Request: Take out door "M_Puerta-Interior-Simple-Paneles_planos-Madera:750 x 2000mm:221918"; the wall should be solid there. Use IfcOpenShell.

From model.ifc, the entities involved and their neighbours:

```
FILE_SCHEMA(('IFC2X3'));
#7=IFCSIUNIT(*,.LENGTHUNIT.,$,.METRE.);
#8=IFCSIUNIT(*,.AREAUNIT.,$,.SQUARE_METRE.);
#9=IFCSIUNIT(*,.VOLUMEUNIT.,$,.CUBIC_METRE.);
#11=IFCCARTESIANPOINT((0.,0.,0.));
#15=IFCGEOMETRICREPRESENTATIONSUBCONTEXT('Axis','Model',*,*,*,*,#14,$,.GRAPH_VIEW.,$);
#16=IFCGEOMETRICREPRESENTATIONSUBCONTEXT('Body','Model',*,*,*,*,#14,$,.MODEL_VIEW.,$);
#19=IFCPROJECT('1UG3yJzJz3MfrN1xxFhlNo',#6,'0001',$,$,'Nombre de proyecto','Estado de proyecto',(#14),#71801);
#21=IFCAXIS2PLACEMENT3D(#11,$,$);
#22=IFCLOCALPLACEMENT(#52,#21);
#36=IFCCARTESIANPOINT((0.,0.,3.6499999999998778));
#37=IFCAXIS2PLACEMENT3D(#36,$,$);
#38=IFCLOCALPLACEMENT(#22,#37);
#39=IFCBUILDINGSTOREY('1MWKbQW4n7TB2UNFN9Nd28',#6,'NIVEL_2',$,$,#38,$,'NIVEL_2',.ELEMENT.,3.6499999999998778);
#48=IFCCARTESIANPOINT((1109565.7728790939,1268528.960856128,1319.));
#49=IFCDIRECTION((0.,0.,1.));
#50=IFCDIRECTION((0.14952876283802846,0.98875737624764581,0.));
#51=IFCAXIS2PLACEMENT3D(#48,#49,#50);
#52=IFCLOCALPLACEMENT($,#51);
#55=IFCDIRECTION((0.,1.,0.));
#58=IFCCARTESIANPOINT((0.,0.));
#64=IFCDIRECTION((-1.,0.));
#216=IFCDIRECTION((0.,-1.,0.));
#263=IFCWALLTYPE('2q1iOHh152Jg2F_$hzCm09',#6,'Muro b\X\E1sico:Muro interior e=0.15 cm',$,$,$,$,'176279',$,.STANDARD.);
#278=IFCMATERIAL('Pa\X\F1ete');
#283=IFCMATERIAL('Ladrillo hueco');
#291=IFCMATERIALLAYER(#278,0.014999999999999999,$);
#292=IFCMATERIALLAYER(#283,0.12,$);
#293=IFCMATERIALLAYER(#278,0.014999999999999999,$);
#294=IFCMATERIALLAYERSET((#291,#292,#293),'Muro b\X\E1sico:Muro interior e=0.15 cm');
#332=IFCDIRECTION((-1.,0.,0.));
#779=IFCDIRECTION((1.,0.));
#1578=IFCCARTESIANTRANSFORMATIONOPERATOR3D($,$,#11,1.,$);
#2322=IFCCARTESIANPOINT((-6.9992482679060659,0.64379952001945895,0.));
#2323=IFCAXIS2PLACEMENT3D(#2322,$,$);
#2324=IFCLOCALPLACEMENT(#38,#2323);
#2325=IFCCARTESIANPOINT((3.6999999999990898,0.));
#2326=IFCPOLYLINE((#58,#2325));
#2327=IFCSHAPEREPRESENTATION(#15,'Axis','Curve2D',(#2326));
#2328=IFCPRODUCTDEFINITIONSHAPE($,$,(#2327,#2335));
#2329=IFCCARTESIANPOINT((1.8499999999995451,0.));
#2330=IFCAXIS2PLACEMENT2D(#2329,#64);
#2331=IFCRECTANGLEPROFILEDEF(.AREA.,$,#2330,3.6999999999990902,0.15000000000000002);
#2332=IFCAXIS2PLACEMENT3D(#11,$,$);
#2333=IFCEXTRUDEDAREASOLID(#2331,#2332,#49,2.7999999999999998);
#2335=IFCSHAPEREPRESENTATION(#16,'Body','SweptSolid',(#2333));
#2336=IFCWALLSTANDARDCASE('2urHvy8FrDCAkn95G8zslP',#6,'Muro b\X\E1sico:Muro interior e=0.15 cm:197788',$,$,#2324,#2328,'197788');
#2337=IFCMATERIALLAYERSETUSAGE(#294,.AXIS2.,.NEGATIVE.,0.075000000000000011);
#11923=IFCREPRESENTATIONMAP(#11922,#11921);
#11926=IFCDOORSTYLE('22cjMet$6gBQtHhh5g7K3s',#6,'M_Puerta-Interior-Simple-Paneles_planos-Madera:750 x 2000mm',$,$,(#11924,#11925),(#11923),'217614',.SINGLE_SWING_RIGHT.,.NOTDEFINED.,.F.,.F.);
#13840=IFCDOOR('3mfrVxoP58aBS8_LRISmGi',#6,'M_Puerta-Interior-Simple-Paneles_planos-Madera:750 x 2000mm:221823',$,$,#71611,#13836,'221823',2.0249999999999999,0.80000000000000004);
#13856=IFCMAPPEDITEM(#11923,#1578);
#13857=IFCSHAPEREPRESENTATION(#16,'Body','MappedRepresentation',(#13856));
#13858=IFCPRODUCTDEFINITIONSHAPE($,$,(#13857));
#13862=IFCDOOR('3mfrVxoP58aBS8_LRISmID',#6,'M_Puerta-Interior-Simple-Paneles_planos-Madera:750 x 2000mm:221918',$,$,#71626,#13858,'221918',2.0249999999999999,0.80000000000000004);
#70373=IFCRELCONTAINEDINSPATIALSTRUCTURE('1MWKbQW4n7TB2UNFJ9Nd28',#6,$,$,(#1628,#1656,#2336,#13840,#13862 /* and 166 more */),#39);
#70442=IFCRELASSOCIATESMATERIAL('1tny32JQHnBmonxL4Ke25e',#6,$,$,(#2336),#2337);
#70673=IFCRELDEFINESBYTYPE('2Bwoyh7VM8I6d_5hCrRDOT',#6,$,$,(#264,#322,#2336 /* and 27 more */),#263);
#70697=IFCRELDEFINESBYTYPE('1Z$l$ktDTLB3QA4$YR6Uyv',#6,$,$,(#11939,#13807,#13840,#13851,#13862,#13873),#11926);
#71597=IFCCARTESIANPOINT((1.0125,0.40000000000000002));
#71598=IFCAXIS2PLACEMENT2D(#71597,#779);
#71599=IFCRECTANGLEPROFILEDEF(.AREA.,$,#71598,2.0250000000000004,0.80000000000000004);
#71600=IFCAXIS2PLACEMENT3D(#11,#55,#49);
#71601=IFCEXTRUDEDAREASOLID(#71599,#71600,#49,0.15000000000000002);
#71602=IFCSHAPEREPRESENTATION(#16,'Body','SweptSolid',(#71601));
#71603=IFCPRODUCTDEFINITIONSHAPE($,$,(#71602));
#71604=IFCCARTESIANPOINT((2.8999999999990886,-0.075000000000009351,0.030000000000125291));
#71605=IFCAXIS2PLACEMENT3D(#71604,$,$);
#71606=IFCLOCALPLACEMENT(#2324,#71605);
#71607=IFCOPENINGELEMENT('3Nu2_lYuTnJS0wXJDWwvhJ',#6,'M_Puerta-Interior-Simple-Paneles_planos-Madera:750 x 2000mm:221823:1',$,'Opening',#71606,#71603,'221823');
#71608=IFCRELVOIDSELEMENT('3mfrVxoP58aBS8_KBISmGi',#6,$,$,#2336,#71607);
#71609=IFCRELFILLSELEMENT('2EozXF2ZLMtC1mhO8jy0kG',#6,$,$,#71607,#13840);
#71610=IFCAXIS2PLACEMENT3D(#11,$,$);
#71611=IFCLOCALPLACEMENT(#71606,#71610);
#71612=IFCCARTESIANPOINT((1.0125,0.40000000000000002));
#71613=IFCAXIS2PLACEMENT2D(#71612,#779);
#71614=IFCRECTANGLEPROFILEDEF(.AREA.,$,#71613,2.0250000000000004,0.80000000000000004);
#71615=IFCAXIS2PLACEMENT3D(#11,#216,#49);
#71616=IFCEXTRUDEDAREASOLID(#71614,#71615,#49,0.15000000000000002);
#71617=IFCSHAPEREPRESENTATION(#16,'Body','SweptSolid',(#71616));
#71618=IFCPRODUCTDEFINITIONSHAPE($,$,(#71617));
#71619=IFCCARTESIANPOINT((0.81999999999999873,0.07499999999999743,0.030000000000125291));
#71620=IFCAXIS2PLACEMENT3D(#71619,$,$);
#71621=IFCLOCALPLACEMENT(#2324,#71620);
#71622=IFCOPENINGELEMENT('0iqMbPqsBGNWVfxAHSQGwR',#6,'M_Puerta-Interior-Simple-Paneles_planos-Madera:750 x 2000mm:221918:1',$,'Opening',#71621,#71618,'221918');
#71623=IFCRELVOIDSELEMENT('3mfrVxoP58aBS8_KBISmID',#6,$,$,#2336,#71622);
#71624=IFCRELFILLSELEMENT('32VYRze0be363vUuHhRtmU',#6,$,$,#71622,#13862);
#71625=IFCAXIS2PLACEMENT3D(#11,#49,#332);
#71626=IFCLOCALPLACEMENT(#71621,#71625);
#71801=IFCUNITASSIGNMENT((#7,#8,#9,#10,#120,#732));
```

```python
import ifcopenshell
import ifcopenshell.api.feature
import ifcopenshell.api.root
import ifcopenshell.geom
import ifcopenshell.util.shape

model = ifcopenshell.open("model.ifc")
settings = ifcopenshell.geom.settings()


def volume(element):
    """Net volume in cubic metres, openings subtracted."""
    shape = ifcopenshell.geom.create_shape(settings, element)
    return ifcopenshell.util.shape.get_volume(shape.geometry)


door = model.by_guid("3mfrVxoP58aBS8_LRISmID")
opening = door.FillsVoids[0].RelatingOpeningElement
wall = opening.VoidsElements[0].RelatingBuildingElement
before = volume(wall)

ifcopenshell.api.root.remove_product(model, product=door)
ifcopenshell.api.feature.remove_feature(model, feature=opening)

after = volume(wall)

print(f"wall volume {before:.3f} -> {after:.3f} m3")

model.write("model_updated.ifc")
```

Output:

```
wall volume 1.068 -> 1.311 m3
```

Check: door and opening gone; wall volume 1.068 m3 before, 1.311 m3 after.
